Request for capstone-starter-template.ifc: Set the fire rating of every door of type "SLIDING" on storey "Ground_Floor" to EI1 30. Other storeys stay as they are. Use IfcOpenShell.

First a look at what the model holds.

```python
import ifcopenshell
import ifcopenshell.util.element

model = ifcopenshell.open("capstone-starter-template.ifc")
print(model.schema)
storey = next(s for s in model.by_type("IfcBuildingStorey") if s.Name == "Ground_Floor")
doors = [e for e in ifcopenshell.util.element.get_decomposition(storey) if e.is_a("IfcDoor")]
seen = {}
for e in doors:
    element_type = ifcopenshell.util.element.get_type(e)
    key = (element_type.Name if element_type != e and element_type else None, ifcopenshell.util.element.get_pset(e, "Pset_DoorCommon", "FireRating"))
    seen[key] = seen.get(key, 0) + 1
for (name, value), count in sorted(seen.items(), key=str):
    print(count, "x", name, "|", value)
```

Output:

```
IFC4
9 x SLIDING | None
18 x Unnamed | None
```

```python
import ifcopenshell
import ifcopenshell.api.pset
import ifcopenshell.util.element

model = ifcopenshell.open("capstone-starter-template.ifc")

storey = next(s for s in model.by_type("IfcBuildingStorey") if s.Name == "Ground_Floor")
doors = [e for e in ifcopenshell.util.element.get_decomposition(storey) if e.is_a("IfcDoor")]

count = 0
for e in doors:
    element_type = ifcopenshell.util.element.get_type(e)
    if element_type in (None, e) or element_type.Name != "SLIDING":
        continue
    # add_pset returns the element's existing set when there is one.
    pset = ifcopenshell.api.pset.add_pset(model, product=e, name="Pset_DoorCommon")
    ifcopenshell.api.pset.edit_pset(model, pset=pset, properties={"FireRating": "EI1 30"})
    count += 1

print(count, "doors updated")

model.write("capstone-starter-template_updated.ifc")
```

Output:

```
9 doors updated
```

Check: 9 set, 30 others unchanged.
